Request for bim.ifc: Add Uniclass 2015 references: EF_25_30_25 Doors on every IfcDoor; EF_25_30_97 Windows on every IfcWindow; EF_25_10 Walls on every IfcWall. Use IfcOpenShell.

First a look at what the model holds.

```python
import ifcopenshell

model = ifcopenshell.open("bim.ifc")
print(model.schema)
print("classifications:", [c.Name for c in model.by_type("IfcClassification")])
for ifc_class in ("IfcDoor", "IfcRoof", "IfcStair", "IfcWall", "IfcWindow"):
    print(ifc_class, len(model.by_type(ifc_class)))
```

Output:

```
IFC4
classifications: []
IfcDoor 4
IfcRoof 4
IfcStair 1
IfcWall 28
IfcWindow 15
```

```python
import ifcopenshell
import ifcopenshell.api.classification

model = ifcopenshell.open("bim.ifc")

system = ifcopenshell.api.classification.add_classification(model, classification="Uniclass 2015")

codes = {
    "IfcDoor": ("EF_25_30_25", "Doors"),
    "IfcWindow": ("EF_25_30_97", "Windows"),
    "IfcWall": ("EF_25_10", "Walls"),
}
for ifc_class, (code, name) in codes.items():
    products = model.by_type(ifc_class)
    ifcopenshell.api.classification.add_reference(
        model, products=products, classification=system, identification=code, name=name
    )
    print(code, len(products))

model.write("bim-out.ifc")
```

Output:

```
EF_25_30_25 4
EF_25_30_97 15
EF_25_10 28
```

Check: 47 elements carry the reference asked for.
